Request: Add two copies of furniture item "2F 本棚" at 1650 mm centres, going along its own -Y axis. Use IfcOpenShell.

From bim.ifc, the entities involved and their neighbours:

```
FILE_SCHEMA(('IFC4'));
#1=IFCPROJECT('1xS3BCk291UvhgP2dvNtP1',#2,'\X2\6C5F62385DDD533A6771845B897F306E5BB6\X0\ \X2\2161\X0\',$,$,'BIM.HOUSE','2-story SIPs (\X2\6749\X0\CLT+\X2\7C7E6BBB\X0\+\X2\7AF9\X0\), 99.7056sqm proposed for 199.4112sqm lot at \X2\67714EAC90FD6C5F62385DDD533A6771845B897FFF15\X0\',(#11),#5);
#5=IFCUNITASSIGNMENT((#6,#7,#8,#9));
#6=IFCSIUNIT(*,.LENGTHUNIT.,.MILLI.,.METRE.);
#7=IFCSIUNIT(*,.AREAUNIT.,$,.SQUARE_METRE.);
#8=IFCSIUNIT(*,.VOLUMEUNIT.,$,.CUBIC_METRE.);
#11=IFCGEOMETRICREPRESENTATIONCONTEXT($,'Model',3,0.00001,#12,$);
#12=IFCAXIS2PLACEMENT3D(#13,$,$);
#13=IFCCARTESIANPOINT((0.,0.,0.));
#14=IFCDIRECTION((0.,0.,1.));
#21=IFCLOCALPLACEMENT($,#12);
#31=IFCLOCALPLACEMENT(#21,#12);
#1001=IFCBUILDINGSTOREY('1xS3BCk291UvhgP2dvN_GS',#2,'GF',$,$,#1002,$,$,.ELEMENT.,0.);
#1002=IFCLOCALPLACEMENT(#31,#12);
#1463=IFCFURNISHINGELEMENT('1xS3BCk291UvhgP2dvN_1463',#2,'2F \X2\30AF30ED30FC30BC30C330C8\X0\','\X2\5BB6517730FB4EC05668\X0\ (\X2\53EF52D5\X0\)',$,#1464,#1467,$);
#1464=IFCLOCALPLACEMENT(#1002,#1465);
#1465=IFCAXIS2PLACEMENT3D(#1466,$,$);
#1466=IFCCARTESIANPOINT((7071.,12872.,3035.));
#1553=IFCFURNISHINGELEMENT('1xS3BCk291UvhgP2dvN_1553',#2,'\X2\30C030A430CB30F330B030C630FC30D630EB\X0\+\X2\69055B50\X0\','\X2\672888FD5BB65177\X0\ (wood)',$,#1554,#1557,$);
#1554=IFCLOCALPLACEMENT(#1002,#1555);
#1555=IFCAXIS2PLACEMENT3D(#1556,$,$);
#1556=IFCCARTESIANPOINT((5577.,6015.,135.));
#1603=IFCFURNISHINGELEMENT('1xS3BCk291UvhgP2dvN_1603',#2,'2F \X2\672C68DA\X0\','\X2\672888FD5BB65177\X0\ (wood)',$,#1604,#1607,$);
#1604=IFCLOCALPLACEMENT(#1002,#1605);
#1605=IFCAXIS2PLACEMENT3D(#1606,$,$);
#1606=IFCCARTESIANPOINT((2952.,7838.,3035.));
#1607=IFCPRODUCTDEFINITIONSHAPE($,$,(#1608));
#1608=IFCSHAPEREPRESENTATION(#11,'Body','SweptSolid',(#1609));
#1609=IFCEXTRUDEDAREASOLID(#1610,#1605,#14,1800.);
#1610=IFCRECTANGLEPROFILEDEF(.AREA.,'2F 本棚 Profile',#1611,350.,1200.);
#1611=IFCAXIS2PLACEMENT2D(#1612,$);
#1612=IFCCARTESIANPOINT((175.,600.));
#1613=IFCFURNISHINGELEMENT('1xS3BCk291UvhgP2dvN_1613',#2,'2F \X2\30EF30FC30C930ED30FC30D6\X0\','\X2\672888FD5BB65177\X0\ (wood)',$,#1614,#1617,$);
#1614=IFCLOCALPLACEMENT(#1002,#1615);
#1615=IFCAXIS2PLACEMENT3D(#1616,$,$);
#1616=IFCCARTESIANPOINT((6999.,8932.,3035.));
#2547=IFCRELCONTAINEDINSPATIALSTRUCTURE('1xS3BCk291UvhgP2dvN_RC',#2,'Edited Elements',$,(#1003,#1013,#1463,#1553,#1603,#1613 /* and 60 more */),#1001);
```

```python
import ifcopenshell
import ifcopenshell.api.geometry
import ifcopenshell.api.root
import ifcopenshell.util.element
import ifcopenshell.util.placement

model = ifcopenshell.open("bim.ifc")


def reuse_history(source, copy):
    """copy_class also copies each property set's owner history, people and application; keep the originals."""
    for rel in copy.IsDefinedBy:
        if rel.is_a("IfcRelDefinesByProperties") and (history := rel.RelatingPropertyDefinition.OwnerHistory):
            rel.RelatingPropertyDefinition.OwnerHistory = source.OwnerHistory
            ifcopenshell.util.element.remove_deep2(model, history)


source = model.by_guid("1xS3BCk291UvhgP2dvN_1603")
base = ifcopenshell.util.placement.get_local_placement(source.ObjectPlacement)
step = -base[:3, 1] * 1650.0

for i in range(1, 3):
    copy = ifcopenshell.api.root.copy_class(model, product=source)
    copy.Representation = ifcopenshell.util.element.copy_deep(
        model, source.Representation, exclude=["IfcGeometricRepresentationContext", "IfcRepresentationMap"]
    )
    reuse_history(source, copy)
    matrix = base.copy()
    matrix[:3, 3] += i * step
    print("added at", matrix[:3, 3].round(3) + 0.0)
    ifcopenshell.api.geometry.edit_object_placement(model, product=copy, matrix=matrix, is_si=False)

model.write("bim_edited.ifc")
```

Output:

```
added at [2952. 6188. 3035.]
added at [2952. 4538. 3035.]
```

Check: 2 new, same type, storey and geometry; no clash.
